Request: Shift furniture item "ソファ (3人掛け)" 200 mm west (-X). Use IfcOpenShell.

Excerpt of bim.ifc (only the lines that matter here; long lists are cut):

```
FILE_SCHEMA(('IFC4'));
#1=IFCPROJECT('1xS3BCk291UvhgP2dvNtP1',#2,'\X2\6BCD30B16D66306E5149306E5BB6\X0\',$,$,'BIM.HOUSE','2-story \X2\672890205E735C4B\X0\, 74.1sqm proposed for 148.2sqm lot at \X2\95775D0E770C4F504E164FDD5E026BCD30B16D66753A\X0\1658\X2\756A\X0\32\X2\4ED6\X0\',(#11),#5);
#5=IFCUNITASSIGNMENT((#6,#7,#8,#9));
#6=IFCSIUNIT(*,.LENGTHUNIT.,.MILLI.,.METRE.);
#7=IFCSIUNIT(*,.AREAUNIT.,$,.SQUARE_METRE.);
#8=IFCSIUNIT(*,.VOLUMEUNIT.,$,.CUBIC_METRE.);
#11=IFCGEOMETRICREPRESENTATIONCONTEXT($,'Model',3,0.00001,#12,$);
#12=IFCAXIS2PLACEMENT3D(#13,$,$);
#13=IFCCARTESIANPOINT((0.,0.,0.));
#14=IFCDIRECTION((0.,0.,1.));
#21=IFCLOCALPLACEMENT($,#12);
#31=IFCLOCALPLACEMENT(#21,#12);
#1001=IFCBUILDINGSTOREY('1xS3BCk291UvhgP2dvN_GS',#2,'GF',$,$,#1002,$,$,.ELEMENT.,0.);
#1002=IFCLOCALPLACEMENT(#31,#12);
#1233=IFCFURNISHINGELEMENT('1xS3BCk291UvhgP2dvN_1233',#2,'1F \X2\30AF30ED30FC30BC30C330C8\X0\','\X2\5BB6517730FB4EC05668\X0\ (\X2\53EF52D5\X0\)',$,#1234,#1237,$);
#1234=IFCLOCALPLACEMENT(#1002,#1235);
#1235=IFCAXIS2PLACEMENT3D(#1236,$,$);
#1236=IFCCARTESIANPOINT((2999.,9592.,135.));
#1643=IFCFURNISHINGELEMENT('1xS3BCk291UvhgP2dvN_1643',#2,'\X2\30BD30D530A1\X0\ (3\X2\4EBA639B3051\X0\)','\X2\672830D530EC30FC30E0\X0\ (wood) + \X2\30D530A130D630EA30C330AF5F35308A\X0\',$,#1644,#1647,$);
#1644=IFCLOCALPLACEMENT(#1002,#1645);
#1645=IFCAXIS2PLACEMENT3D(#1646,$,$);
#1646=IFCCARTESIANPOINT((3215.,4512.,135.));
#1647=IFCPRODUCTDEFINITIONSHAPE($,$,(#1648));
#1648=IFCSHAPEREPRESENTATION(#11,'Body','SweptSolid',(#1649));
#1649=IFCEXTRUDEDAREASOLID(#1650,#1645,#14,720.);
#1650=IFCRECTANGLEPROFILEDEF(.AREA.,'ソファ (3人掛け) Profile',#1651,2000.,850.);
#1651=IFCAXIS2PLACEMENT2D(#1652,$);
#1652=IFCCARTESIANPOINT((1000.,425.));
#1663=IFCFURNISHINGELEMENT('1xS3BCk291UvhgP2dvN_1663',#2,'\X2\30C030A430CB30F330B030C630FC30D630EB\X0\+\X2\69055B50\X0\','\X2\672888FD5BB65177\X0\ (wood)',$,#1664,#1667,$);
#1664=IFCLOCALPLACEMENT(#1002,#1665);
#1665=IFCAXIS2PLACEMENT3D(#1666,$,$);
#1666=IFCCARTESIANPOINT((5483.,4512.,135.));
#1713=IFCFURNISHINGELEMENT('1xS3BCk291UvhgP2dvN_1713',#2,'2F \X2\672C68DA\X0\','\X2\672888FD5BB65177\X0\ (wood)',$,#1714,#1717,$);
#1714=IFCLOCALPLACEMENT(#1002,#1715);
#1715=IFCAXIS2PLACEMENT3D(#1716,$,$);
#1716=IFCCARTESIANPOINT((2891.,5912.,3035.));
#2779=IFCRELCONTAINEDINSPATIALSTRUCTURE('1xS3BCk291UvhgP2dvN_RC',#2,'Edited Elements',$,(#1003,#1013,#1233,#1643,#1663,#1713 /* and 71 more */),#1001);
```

```python
import ifcopenshell
import ifcopenshell.api.geometry
import ifcopenshell.util.placement
import ifcopenshell.util.unit

model = ifcopenshell.open("bim.ifc")
unit_scale = ifcopenshell.util.unit.calculate_unit_scale(model)

item = model.by_guid("1xS3BCk291UvhgP2dvN_1643")
matrix = ifcopenshell.util.placement.get_local_placement(item.ObjectPlacement)
matrix[0, 3] -= 0.2 / unit_scale
ifcopenshell.api.geometry.edit_object_placement(model, product=item, matrix=matrix, is_si=False)

print(ifcopenshell.util.placement.get_local_placement(item.ObjectPlacement).round(3) + 0.0)

model.write("bim_edited.ifc")
```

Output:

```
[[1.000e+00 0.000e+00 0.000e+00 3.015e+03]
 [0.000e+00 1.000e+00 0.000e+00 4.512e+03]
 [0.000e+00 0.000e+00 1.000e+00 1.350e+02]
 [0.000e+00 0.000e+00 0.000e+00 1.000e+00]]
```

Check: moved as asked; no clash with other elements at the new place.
